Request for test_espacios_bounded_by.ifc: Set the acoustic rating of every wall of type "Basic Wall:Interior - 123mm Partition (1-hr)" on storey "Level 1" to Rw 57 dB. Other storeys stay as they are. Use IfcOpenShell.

First a look at what the model holds.

```python
import ifcopenshell
import ifcopenshell.util.element

model = ifcopenshell.open("test_espacios_bounded_by.ifc")
print(model.schema)
storey = next(s for s in model.by_type("IfcBuildingStorey") if s.Name == "Level 1")
walls = [e for e in ifcopenshell.util.element.get_decomposition(storey) if e.is_a("IfcWall")]
seen = {}
for e in walls:
    element_type = ifcopenshell.util.element.get_type(e)
    key = (element_type.Name if element_type != e and element_type else None, ifcopenshell.util.element.get_pset(e, "Pset_WallCommon", "AcousticRating"))
    seen[key] = seen.get(key, 0) + 1
for (name, value), count in sorted(seen.items(), key=str):
    print(count, "x", name, "|", value)
```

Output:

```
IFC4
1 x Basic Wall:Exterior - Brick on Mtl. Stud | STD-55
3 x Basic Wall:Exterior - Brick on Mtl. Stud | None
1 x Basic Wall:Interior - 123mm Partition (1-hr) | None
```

```python
import ifcopenshell
import ifcopenshell.api.pset
import ifcopenshell.util.element

model = ifcopenshell.open("test_espacios_bounded_by.ifc")

storey = next(s for s in model.by_type("IfcBuildingStorey") if s.Name == "Level 1")
walls = [e for e in ifcopenshell.util.element.get_decomposition(storey) if e.is_a("IfcWall")]

count = 0
for e in walls:
    element_type = ifcopenshell.util.element.get_type(e)
    if element_type in (None, e) or element_type.Name != "Basic Wall:Interior - 123mm Partition (1-hr)":
        continue
    # add_pset returns the element's existing set when there is one.
    pset = ifcopenshell.api.pset.add_pset(model, product=e, name="Pset_WallCommon")
    ifcopenshell.api.pset.edit_pset(model, pset=pset, properties={"AcousticRating": "Rw 57 dB"})
    count += 1

print(count, "walls updated")

model.write("test_espacios_bounded_by-out.ifc")
```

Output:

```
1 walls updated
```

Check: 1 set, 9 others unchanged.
